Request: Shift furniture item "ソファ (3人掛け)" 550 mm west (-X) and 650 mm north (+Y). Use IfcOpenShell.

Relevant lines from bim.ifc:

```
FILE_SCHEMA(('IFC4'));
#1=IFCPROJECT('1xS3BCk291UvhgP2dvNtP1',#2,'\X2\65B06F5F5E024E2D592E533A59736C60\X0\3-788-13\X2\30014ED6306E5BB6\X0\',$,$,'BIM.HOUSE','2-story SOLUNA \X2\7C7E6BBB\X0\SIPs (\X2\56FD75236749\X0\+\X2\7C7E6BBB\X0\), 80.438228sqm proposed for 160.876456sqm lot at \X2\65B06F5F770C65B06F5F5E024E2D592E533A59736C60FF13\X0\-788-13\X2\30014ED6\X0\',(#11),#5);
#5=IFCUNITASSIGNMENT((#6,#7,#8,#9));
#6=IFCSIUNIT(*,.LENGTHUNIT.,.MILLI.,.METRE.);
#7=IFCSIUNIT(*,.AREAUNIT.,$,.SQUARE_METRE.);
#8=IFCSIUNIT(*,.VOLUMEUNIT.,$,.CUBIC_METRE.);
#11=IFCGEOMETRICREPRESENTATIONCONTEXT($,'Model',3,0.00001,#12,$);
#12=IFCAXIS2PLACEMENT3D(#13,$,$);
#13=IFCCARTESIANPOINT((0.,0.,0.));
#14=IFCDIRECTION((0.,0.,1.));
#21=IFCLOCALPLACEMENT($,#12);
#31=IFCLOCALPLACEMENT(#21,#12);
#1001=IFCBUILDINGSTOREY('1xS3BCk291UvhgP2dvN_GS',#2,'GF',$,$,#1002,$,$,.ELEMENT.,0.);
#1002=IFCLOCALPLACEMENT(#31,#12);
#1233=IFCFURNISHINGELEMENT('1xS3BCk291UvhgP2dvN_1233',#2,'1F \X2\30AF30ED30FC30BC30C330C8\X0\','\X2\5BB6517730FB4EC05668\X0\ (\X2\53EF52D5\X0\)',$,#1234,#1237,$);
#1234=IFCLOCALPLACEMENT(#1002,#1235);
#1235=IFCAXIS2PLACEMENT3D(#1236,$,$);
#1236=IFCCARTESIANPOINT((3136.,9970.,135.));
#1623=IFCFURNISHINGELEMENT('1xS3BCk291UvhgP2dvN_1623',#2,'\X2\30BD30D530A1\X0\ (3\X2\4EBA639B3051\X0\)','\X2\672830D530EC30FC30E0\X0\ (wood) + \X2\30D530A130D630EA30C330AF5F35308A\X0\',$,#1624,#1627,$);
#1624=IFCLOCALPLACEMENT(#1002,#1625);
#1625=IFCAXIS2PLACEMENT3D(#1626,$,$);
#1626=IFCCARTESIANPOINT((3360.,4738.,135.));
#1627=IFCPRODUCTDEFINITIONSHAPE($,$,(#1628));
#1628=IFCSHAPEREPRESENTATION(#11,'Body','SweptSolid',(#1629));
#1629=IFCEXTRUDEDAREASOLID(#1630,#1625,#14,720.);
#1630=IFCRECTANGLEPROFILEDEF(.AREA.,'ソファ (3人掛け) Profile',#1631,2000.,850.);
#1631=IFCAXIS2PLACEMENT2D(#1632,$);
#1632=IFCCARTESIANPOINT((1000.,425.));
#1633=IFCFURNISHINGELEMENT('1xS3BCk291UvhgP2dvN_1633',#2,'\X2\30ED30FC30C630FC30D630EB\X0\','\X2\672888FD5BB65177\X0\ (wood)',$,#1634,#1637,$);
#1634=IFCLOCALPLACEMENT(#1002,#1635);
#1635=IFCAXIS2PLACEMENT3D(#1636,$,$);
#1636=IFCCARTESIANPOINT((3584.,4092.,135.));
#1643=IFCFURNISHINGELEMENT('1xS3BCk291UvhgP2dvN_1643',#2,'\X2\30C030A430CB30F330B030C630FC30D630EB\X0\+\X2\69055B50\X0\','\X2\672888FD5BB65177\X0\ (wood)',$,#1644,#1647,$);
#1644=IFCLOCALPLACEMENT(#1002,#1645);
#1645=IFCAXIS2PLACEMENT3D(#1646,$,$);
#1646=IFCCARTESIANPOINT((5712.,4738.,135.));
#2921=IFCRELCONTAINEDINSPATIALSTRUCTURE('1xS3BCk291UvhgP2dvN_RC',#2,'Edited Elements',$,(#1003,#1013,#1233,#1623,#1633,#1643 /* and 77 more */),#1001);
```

```python
import ifcopenshell
import ifcopenshell.api.geometry
import ifcopenshell.util.placement

model = ifcopenshell.open("bim.ifc")

item = model.by_id(1623)
matrix = ifcopenshell.util.placement.get_local_placement(item.ObjectPlacement)
matrix[0, 3] -= 550.0
matrix[1, 3] += 650.0
ifcopenshell.api.geometry.edit_object_placement(model, product=item, matrix=matrix, is_si=False)

print(ifcopenshell.util.placement.get_local_placement(item.ObjectPlacement).round(3) + 0.0)

model.write("bim_rev.ifc")
```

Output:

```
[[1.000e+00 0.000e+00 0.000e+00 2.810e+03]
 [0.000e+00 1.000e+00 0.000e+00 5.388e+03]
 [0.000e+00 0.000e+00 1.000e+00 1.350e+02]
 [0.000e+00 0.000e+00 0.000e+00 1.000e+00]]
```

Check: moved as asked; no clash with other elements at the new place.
